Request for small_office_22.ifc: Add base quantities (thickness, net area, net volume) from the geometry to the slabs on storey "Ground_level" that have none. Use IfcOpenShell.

First a look at what the model holds.

```python
import ifcopenshell
import ifcopenshell.util.element
import ifcopenshell.util.unit

model = ifcopenshell.open("small_office_22.ifc")
print(model.schema)
for unit_type in ("LENGTHUNIT", "AREAUNIT", "VOLUMEUNIT"):
    print(unit_type, ifcopenshell.util.unit.calculate_unit_scale(model, unit_type))
storey = next(s for s in model.by_type("IfcBuildingStorey") if s.Name == "Ground_level")
slabs = [e for e in ifcopenshell.util.element.get_decomposition(storey) if e.is_a("IfcSlab")]
for e in sorted(slabs, key=lambda e: e.id()):
    print(e.id(), e.is_a(), e.Name, list(ifcopenshell.util.element.get_psets(e, qtos_only=True)), sep=" | ")
```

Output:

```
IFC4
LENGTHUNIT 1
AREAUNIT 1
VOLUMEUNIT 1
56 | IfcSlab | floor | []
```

```python
import ifcopenshell
import ifcopenshell.api.pset
import ifcopenshell.geom
import ifcopenshell.util.element
import ifcopenshell.util.shape
import ifcopenshell.util.unit

model = ifcopenshell.open("small_office_22.ifc")
unit_scale = ifcopenshell.util.unit.calculate_unit_scale(model)
area_scale = ifcopenshell.util.unit.calculate_unit_scale(model, "AREAUNIT")
volume_scale = ifcopenshell.util.unit.calculate_unit_scale(model, "VOLUMEUNIT")
settings = ifcopenshell.geom.settings()

storey = next(s for s in model.by_type("IfcBuildingStorey") if s.Name == "Ground_level")
slabs = [e for e in ifcopenshell.util.element.get_decomposition(storey) if e.is_a("IfcSlab")]

for e in sorted(slabs, key=lambda e: e.id()):
    if ifcopenshell.util.element.get_psets(e, qtos_only=True, should_inherit=False):
        continue
    # Geometry comes back in metres, in the element's own axes.
    shape = ifcopenshell.geom.create_shape(settings, e)
    values = {
        "Width": ifcopenshell.util.shape.get_z(shape.geometry) / unit_scale,
        "NetArea": ifcopenshell.util.shape.get_footprint_area(shape.geometry) / area_scale,
        "NetVolume": ifcopenshell.util.shape.get_volume(shape.geometry) / volume_scale,
    }
    qto = ifcopenshell.api.pset.add_qto(model, product=e, name="Qto_SlabBaseQuantities")
    ifcopenshell.api.pset.edit_qto(model, qto=qto, properties=values)
    print(e.id(), {k: round(v, 3) for k, v in values.items()})

model.write("small_office_22_rev.ifc")
```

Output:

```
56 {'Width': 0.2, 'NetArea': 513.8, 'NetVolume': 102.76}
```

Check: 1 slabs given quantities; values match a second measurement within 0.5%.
